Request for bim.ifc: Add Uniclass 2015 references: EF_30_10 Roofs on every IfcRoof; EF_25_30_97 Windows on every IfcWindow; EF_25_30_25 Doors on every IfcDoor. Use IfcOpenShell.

First a look at what the model holds.

```python
import ifcopenshell

model = ifcopenshell.open("bim.ifc")
print(model.schema)
print("classifications:", [c.Name for c in model.by_type("IfcClassification")])
for ifc_class in ("IfcDoor", "IfcRoof", "IfcStair", "IfcWall", "IfcWindow"):
    print(ifc_class, len(model.by_type(ifc_class)))
```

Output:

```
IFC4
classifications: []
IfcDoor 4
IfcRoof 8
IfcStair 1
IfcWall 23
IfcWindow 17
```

```python
import ifcopenshell
import ifcopenshell.api.classification

model = ifcopenshell.open("bim.ifc")

system = ifcopenshell.api.classification.add_classification(model, classification="Uniclass 2015")

codes = {
    "IfcRoof": ("EF_30_10", "Roofs"),
    "IfcWindow": ("EF_25_30_97", "Windows"),
    "IfcDoor": ("EF_25_30_25", "Doors"),
}
for ifc_class, (code, name) in codes.items():
    products = model.by_type(ifc_class)
    ifcopenshell.api.classification.add_reference(
        model, products=products, classification=system, identification=code, name=name
    )
    print(code, len(products))

model.write("bim_rev.ifc")
```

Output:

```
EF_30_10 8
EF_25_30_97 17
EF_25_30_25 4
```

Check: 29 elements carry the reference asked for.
